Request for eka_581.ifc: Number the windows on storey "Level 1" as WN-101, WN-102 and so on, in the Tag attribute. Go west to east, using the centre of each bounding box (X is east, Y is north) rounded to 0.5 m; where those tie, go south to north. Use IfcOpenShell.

First a look at what the model holds.

```python
import ifcopenshell
import ifcopenshell.util.element
import ifcopenshell.util.placement

model = ifcopenshell.open("eka_581.ifc")
print(model.schema)
storey = next(s for s in model.by_type("IfcBuildingStorey") if s.Name == "Level 1")
windows = [e for e in ifcopenshell.util.element.get_decomposition(storey) if e.is_a("IfcWindow")]
for e in sorted(windows, key=lambda e: e.id()):
    origin = ifcopenshell.util.placement.get_local_placement(e.ObjectPlacement)[:3, 3]
    print(e.id(), e.Tag, e.Name, origin.round(2) + 0.0, sep=" | ")
```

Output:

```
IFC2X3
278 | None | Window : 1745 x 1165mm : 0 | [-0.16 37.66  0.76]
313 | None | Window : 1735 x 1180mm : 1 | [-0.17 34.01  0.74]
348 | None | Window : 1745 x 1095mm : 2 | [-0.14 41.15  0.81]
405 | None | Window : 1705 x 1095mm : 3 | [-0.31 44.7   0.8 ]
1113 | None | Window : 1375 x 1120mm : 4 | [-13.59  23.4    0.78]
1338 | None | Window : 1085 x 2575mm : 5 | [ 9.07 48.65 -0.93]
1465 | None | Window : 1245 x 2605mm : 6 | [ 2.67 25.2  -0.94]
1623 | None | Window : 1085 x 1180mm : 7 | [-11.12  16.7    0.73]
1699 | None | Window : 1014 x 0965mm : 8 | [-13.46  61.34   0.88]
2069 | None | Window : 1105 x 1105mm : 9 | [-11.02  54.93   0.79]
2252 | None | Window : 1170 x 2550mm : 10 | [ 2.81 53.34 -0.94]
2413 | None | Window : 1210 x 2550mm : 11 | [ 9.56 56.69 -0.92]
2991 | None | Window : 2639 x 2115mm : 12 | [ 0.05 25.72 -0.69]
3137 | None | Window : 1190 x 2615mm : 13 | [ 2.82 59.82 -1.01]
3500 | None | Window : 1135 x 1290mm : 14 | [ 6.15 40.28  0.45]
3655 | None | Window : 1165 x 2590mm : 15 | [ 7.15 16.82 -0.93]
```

```python
import ifcopenshell
import ifcopenshell.geom
import ifcopenshell.util.element
import ifcopenshell.util.shape

model = ifcopenshell.open("eka_581.ifc")
settings = ifcopenshell.geom.settings()
settings.set("use-world-coords", True)


def centre(element):
    shape = ifcopenshell.geom.create_shape(settings, element)
    return ifcopenshell.util.shape.get_bbox_centroid(shape.geometry)


storey = next(s for s in model.by_type("IfcBuildingStorey") if s.Name == "Level 1")
windows = [e for e in ifcopenshell.util.element.get_decomposition(storey) if e.is_a("IfcWindow")]

# Insertion points can sit at a corner or the storey origin, so sort by the geometry (in metres).
centres = {e: centre(e) for e in windows}
windows.sort(key=lambda e: (round(centres[e][0] / 0.5), centres[e][1]))

for i, e in enumerate(windows, start=1):
    number = f"WN-1{i:02d}"
    e.Tag = number
    print(e.id(), number)

model.write("eka_581_v2.ifc")
```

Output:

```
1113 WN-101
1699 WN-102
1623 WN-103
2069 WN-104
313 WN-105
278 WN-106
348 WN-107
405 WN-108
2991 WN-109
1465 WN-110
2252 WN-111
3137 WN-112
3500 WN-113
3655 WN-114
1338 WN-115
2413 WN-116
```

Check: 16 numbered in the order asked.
